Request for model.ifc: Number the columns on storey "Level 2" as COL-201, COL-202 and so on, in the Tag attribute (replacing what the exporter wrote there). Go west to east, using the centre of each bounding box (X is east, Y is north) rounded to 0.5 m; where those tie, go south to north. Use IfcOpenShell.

First a look at what the model holds.

```python
import ifcopenshell
import ifcopenshell.util.element
import ifcopenshell.util.placement

model = ifcopenshell.open("model.ifc")
print(model.schema)
storey = next(s for s in model.by_type("IfcBuildingStorey") if s.Name == "Level 2")
columns = [e for e in ifcopenshell.util.element.get_decomposition(storey) if e.is_a("IfcColumn")]
for e in sorted(columns, key=lambda e: e.id()):
    origin = ifcopenshell.util.placement.get_local_placement(e.ObjectPlacement)[:3, 3]
    print(e.id(), e.Tag, e.Name, origin.round(2) + 0.0, sep=" | ")
```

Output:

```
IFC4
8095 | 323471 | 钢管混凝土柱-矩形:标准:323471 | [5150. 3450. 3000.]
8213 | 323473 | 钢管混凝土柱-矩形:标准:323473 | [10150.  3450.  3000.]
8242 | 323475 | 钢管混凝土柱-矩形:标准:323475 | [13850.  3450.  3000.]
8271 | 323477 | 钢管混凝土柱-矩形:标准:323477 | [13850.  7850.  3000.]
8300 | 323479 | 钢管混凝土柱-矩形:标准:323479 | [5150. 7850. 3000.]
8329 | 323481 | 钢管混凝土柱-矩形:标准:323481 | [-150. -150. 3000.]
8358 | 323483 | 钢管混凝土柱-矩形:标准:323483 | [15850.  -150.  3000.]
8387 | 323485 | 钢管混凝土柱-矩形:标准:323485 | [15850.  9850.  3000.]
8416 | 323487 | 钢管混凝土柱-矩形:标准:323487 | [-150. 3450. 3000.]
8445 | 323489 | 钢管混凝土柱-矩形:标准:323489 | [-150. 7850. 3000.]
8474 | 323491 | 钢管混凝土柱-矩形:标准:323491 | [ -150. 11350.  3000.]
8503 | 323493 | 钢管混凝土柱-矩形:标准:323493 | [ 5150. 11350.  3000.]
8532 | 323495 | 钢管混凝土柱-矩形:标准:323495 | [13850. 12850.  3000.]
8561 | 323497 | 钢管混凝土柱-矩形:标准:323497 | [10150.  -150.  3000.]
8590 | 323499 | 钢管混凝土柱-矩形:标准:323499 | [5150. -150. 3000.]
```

```python
import ifcopenshell
import ifcopenshell.geom
import ifcopenshell.util.element
import ifcopenshell.util.shape

model = ifcopenshell.open("model.ifc")
settings = ifcopenshell.geom.settings()
settings.set("use-world-coords", True)


def centre(element):
    shape = ifcopenshell.geom.create_shape(settings, element)
    return ifcopenshell.util.shape.get_bbox_centroid(shape.geometry)


storey = next(s for s in model.by_type("IfcBuildingStorey") if s.Name == "Level 2")
columns = [e for e in ifcopenshell.util.element.get_decomposition(storey) if e.is_a("IfcColumn")]

# Insertion points can sit at a corner or the storey origin, so sort by the geometry (in metres).
centres = {e: centre(e) for e in columns}
columns.sort(key=lambda e: (round(centres[e][0] / 0.5), centres[e][1]))

for i, e in enumerate(columns, start=1):
    number = f"COL-2{i:02d}"
    e.Tag = number
    print(e.id(), number)

model.write("model_updated.ifc")
```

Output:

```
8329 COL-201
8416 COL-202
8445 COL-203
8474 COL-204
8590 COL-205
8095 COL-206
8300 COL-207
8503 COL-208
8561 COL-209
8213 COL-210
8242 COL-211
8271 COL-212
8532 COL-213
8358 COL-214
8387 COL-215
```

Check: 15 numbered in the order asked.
